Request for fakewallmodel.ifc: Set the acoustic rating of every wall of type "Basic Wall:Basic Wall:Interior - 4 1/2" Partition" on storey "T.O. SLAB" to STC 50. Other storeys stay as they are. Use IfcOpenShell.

First a look at what the model holds.

```python
import ifcopenshell
import ifcopenshell.util.element

model = ifcopenshell.open("fakewallmodel.ifc")
print(model.schema)
storey = next(s for s in model.by_type("IfcBuildingStorey") if s.Name == "T.O. SLAB")
walls = [e for e in ifcopenshell.util.element.get_decomposition(storey) if e.is_a("IfcWall")]
seen = {}
for e in walls:
    element_type = ifcopenshell.util.element.get_type(e)
    key = (element_type.Name if element_type != e and element_type else None, ifcopenshell.util.element.get_pset(e, "Pset_WallCommon", "AcousticRating"))
    seen[key] = seen.get(key, 0) + 1
for (name, value), count in sorted(seen.items(), key=str):
    print(count, "x", name, "|", value)
```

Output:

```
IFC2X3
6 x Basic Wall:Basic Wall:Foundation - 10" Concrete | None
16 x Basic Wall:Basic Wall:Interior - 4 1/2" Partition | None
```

```python
import ifcopenshell
import ifcopenshell.api.pset
import ifcopenshell.util.element

model = ifcopenshell.open("fakewallmodel.ifc")

storey = next(s for s in model.by_type("IfcBuildingStorey") if s.Name == "T.O. SLAB")
walls = [e for e in ifcopenshell.util.element.get_decomposition(storey) if e.is_a("IfcWall")]

count = 0
for e in walls:
    element_type = ifcopenshell.util.element.get_type(e)
    if element_type in (None, e) or element_type.Name != 'Basic Wall:Basic Wall:Interior - 4 1/2" Partition':
        continue
    # add_pset returns the element's existing set when there is one.
    pset = ifcopenshell.api.pset.add_pset(model, product=e, name="Pset_WallCommon")
    ifcopenshell.api.pset.edit_pset(model, pset=pset, properties={"AcousticRating": "STC 50"})
    count += 1

print(count, "walls updated")

model.write("fakewallmodel-out.ifc")
```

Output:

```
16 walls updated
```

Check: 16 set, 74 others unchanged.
